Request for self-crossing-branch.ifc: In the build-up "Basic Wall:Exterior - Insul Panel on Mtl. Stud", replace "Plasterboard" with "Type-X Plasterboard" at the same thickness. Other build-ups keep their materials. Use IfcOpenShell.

First a look at what the model holds.

```python
import ifcopenshell
import ifcopenshell.util.element

model = ifcopenshell.open("self-crossing-branch.ifc")
print(model.schema)
for layer_set in model.by_type("IfcMaterialLayerSet"):
    if layer_set.LayerSetName == "Basic Wall:Exterior - Insul Panel on Mtl. Stud":
        for layer in layer_set.MaterialLayers:
            print(layer.id(), layer.Material and layer.Material.Name, layer.LayerThickness, sep=" | ")
        print(len(ifcopenshell.util.element.get_elements_by_material(model, layer_set)), "elements and types use it")
print(sorted(m.Name for m in model.by_type("IfcMaterial") if m.Name)[:60])
```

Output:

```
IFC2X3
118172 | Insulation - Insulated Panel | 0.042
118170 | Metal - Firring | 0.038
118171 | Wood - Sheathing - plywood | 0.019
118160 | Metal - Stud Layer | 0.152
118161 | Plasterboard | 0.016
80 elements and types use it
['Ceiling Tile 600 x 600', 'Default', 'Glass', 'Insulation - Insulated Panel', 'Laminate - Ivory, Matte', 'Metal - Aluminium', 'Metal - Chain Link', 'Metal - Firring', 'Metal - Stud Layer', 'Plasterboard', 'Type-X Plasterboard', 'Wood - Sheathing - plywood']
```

```python
import ifcopenshell
import ifcopenshell.api.material

model = ifcopenshell.open("self-crossing-branch.ifc")

layer_set = next(s for s in model.by_type("IfcMaterialLayerSet") if s.LayerSetName == "Basic Wall:Exterior - Insul Panel on Mtl. Stud")
layer = next(l for l in layer_set.MaterialLayers if l.Material and l.Material.Name == "Plasterboard")
material = next(m for m in model.by_type("IfcMaterial") if m.Name == "Type-X Plasterboard")

# Point this one layer at the other material; renaming the old one would change it everywhere.
ifcopenshell.api.material.edit_layer(model, layer=layer, attributes={}, material=material)

print([l.Material.Name if l.Material else None for l in layer_set.MaterialLayers])

model.write("self-crossing-branch-out.ifc")
```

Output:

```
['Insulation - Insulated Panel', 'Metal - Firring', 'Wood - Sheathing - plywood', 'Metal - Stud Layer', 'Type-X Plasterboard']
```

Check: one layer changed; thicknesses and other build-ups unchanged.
